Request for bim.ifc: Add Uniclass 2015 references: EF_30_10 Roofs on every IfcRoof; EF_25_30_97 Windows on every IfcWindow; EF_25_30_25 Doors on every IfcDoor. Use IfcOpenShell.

First a look at what the model holds.

```python
import ifcopenshell

model = ifcopenshell.open("bim.ifc")
print(model.schema)
print("classifications:", [c.Name for c in model.by_type("IfcClassification")])
for ifc_class in ("IfcDoor", "IfcRoof", "IfcStair", "IfcWall", "IfcWindow"):
    print(ifc_class, len(model.by_type(ifc_class)))
```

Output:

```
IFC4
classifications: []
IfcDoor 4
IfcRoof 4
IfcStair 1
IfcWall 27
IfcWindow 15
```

```python
import ifcopenshell
import ifcopenshell.api.classification

model = ifcopenshell.open("bim.ifc")

system = ifcopenshell.api.classification.add_classification(model, classification="Uniclass 2015")

codes = {
    "IfcRoof": ("EF_30_10", "Roofs"),
    "IfcWindow": ("EF_25_30_97", "Windows"),
    "IfcDoor": ("EF_25_30_25", "Doors"),
}
for ifc_class, (code, name) in codes.items():
    products = model.by_type(ifc_class)
    ifcopenshell.api.classification.add_reference(
        model, products=products, classification=system, identification=code, name=name
    )
    print(code, len(products))

model.write("bim_rev.ifc")
```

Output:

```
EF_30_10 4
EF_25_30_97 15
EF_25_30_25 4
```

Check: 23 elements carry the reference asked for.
